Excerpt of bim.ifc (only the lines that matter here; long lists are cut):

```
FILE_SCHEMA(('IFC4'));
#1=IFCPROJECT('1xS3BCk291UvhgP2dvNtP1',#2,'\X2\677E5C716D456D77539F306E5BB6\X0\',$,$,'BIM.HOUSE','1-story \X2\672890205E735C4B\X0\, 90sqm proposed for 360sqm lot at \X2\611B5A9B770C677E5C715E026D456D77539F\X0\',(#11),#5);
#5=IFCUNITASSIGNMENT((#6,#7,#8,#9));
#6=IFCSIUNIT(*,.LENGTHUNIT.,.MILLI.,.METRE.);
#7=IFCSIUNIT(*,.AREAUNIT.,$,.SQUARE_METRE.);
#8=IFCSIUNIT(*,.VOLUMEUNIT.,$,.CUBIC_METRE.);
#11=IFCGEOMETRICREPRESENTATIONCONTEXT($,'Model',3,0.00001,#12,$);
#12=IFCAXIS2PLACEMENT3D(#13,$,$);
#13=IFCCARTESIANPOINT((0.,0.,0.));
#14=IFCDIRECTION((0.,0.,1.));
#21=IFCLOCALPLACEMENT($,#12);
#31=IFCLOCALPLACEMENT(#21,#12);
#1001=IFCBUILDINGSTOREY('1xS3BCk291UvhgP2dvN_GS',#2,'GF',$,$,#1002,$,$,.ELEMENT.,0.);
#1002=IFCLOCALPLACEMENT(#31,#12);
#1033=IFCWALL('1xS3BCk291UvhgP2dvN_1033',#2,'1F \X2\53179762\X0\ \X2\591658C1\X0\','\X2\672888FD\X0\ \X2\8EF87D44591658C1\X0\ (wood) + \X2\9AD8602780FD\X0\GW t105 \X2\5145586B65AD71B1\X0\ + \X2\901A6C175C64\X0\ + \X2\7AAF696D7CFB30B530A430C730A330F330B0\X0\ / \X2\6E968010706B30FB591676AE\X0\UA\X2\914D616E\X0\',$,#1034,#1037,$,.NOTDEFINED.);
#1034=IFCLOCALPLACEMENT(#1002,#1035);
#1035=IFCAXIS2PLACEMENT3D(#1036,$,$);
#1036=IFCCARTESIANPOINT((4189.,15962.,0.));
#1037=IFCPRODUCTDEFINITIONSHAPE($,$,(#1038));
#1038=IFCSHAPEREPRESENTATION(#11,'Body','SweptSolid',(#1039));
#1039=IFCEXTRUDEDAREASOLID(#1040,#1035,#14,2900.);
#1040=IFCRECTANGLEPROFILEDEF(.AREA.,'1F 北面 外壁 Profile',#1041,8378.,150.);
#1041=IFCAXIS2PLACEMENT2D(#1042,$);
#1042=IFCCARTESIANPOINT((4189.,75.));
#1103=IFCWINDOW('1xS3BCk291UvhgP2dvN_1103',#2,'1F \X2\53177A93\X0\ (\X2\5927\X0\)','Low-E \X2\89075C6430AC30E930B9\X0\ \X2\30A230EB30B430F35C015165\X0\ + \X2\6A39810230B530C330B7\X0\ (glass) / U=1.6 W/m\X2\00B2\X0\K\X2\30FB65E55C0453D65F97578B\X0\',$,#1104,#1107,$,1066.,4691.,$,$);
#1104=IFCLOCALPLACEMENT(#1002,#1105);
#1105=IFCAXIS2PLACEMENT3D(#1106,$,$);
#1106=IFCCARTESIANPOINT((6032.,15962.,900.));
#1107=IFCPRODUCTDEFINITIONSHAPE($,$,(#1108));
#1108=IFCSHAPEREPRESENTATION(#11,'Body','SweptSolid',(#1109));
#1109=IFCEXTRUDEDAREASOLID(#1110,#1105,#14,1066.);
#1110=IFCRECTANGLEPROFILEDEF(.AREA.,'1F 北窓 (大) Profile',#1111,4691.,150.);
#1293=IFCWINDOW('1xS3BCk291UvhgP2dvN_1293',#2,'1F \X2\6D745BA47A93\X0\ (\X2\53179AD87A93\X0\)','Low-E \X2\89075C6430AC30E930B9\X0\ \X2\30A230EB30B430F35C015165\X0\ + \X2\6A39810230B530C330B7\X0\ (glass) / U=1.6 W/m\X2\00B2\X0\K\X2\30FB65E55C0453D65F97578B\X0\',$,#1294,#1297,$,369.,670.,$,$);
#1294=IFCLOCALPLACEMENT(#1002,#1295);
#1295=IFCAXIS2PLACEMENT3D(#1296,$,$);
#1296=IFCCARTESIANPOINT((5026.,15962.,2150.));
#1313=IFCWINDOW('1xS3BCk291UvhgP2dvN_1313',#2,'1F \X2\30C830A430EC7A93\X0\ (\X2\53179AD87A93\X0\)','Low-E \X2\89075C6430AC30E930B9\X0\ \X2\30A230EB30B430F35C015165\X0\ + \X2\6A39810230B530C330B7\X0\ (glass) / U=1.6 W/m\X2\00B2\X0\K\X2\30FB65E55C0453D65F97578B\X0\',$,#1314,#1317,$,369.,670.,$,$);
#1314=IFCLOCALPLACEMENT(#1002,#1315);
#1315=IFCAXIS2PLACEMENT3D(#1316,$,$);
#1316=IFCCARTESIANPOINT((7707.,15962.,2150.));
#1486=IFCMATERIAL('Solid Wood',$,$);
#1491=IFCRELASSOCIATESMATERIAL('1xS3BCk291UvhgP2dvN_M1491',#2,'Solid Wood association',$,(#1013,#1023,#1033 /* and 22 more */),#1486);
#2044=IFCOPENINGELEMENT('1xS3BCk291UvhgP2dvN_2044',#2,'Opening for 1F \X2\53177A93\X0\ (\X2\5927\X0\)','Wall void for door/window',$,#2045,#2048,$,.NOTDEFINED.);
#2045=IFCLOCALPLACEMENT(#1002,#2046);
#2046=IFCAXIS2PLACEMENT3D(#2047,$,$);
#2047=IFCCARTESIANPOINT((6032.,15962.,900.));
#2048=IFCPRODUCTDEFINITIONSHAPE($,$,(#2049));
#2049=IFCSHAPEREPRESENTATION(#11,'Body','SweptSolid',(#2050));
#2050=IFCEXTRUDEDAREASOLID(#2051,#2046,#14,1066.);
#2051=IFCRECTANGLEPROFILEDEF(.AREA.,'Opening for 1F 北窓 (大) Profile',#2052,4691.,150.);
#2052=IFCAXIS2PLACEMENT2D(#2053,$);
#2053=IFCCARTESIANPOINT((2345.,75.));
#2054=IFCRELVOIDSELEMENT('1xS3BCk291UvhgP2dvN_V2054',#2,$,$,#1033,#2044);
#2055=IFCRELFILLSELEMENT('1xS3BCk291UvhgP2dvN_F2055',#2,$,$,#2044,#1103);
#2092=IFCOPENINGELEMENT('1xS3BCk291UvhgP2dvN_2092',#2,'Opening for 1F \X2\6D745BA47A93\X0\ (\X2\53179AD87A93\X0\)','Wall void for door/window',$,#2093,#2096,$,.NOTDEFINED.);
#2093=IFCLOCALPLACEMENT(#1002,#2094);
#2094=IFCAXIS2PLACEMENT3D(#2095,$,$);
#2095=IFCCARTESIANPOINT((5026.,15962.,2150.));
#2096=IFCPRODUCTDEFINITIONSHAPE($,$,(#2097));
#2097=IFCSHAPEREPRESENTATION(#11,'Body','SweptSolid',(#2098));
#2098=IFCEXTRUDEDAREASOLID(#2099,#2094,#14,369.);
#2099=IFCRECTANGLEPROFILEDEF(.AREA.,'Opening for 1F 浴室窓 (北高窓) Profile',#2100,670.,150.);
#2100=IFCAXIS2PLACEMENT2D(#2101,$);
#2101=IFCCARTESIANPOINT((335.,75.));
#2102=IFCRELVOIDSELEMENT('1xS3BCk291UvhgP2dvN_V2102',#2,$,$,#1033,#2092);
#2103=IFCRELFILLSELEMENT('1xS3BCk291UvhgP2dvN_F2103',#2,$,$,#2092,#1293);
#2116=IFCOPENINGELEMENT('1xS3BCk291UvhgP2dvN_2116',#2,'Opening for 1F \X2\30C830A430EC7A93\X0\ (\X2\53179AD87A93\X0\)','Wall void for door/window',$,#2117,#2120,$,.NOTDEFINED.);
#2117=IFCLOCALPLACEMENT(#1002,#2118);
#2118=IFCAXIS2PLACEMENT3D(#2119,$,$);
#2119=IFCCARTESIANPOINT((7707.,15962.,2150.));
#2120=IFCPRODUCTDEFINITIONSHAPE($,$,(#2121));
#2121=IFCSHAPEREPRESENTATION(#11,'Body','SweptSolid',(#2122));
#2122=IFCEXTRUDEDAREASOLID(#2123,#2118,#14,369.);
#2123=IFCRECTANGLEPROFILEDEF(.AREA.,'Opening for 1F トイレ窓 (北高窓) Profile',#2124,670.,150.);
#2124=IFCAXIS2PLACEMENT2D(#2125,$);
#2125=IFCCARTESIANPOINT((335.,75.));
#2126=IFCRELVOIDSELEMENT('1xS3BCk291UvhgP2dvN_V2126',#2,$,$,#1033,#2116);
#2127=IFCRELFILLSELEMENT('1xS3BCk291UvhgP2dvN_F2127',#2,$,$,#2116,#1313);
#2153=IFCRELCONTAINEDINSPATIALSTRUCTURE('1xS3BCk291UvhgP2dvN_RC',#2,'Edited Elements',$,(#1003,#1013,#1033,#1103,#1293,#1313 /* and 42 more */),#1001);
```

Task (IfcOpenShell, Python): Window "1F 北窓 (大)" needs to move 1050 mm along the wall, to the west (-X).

```python
import ifcopenshell
import ifcopenshell.api.geometry
import ifcopenshell.util.placement
import ifcopenshell.util.unit

model = ifcopenshell.open("bim.ifc")
unit_scale = ifcopenshell.util.unit.calculate_unit_scale(model)

window = model.by_guid("1xS3BCk291UvhgP2dvN_1103")
opening = window.FillsVoids[0].RelatingOpeningElement
wall = opening.VoidsElements[0].RelatingBuildingElement

wall_matrix = ifcopenshell.util.placement.get_local_placement(wall.ObjectPlacement)
shift = wall_matrix[:3, 0] * -1.05 / unit_scale
before = ifcopenshell.util.placement.get_local_placement(window.ObjectPlacement)[:3, 3].copy()

# The window is not placed relative to its opening, so move both.
for product in (opening, window):
    matrix = ifcopenshell.util.placement.get_local_placement(product.ObjectPlacement)
    matrix[:3, 3] += shift
    ifcopenshell.api.geometry.edit_object_placement(model, product=product, matrix=matrix, is_si=False)

after = ifcopenshell.util.placement.get_local_placement(window.ObjectPlacement)[:3, 3]
print("window moved by", (after - before).round(3) + 0.0)

model.write("bim_v2.ifc")
```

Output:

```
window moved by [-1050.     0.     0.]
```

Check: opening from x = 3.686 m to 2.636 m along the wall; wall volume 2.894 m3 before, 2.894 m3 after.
